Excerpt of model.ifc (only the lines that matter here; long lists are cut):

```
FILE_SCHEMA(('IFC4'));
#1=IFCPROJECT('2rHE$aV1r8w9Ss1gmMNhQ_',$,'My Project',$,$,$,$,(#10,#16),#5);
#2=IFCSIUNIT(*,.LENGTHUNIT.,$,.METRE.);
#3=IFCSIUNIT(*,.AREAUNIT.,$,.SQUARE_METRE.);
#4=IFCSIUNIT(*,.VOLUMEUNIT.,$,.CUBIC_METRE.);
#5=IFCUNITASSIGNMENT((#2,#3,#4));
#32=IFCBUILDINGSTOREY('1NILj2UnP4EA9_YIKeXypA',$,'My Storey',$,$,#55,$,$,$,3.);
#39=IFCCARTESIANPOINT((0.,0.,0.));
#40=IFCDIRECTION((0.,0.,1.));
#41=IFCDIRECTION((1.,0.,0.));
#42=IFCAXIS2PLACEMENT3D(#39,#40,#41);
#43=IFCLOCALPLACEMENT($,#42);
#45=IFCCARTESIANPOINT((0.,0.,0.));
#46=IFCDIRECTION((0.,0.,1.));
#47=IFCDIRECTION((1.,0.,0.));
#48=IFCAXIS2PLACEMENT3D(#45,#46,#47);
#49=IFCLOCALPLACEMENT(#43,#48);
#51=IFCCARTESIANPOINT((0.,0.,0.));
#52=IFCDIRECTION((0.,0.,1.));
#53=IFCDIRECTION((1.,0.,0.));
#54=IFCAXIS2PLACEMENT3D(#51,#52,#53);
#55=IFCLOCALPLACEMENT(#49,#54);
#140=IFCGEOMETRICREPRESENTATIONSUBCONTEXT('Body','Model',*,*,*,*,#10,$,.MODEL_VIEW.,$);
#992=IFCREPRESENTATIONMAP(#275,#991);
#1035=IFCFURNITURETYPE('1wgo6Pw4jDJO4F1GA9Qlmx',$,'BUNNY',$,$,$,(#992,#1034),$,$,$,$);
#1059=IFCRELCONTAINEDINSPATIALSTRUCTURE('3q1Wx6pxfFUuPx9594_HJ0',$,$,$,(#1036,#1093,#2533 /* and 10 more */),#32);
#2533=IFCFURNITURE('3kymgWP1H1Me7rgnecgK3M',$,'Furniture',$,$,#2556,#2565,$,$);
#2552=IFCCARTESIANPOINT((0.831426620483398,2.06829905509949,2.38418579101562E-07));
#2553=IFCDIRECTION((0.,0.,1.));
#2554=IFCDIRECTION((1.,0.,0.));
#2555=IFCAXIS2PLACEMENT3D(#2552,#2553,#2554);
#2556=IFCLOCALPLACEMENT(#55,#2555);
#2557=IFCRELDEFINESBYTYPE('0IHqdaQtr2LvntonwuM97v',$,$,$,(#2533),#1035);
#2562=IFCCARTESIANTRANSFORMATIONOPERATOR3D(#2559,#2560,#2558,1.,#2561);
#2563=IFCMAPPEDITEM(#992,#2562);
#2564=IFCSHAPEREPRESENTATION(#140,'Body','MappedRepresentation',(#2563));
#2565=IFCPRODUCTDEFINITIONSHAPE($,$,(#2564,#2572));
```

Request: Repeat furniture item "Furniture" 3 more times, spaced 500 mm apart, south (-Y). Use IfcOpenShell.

```python
import numpy as np
import ifcopenshell
import ifcopenshell.api.geometry
import ifcopenshell.api.root
import ifcopenshell.util.element
import ifcopenshell.util.placement
import ifcopenshell.util.unit

model = ifcopenshell.open("model.ifc")
unit_scale = ifcopenshell.util.unit.calculate_unit_scale(model)

source = model.by_id(2533)
base = ifcopenshell.util.placement.get_local_placement(source.ObjectPlacement)
step = np.array([0.0, -1.0, 0.0]) * 0.5 / unit_scale

for i in range(1, 4):
    copy = ifcopenshell.api.root.copy_class(model, product=source)
    copy.Representation = ifcopenshell.util.element.copy_deep(
        model, source.Representation, exclude=["IfcGeometricRepresentationContext", "IfcRepresentationMap"]
    )
    matrix = base.copy()
    matrix[:3, 3] += i * step
    print("added at", matrix[:3, 3].round(3) + 0.0)
    ifcopenshell.api.geometry.edit_object_placement(model, product=copy, matrix=matrix, is_si=False)

model.write("model_edited.ifc")
```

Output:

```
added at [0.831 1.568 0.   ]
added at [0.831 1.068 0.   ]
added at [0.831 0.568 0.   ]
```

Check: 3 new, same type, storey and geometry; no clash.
